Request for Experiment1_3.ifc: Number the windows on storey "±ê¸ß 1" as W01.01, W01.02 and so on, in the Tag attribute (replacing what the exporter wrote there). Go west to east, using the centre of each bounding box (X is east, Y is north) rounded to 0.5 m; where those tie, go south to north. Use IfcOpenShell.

First a look at what the model holds.

```python
import ifcopenshell
import ifcopenshell.util.element
import ifcopenshell.util.placement

model = ifcopenshell.open("Experiment1_3.ifc")
print(model.schema)
storey = next(s for s in model.by_type("IfcBuildingStorey") if s.Name == "±ê¸ß 1")
windows = [e for e in ifcopenshell.util.element.get_decomposition(storey) if e.is_a("IfcWindow")]
for e in sorted(windows, key=lambda e: e.id()):
    origin = ifcopenshell.util.placement.get_local_placement(e.ObjectPlacement)[:3, 3]
    print(e.id(), e.Tag, e.Name, origin.round(2) + 0.0, sep=" | ")
```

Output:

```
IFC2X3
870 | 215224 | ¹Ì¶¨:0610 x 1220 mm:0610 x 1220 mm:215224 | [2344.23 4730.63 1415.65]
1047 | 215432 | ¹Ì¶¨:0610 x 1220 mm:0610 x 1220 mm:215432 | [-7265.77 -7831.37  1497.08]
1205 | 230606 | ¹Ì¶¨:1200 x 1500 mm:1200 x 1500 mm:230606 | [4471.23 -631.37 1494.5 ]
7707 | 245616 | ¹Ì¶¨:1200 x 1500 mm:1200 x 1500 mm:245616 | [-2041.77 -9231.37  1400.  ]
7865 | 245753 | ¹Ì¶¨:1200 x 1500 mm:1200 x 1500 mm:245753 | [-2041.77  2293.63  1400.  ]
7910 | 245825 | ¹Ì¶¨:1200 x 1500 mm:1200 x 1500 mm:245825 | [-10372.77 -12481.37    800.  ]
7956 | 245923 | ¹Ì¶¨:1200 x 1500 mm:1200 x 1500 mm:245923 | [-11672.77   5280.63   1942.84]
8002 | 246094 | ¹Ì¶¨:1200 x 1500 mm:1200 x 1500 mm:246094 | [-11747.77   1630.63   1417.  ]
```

```python
import ifcopenshell
import ifcopenshell.geom
import ifcopenshell.util.element
import ifcopenshell.util.shape

model = ifcopenshell.open("Experiment1_3.ifc")
settings = ifcopenshell.geom.settings()
settings.set("use-world-coords", True)


def centre(element):
    shape = ifcopenshell.geom.create_shape(settings, element)
    return ifcopenshell.util.shape.get_bbox_centroid(shape.geometry)


storey = next(s for s in model.by_type("IfcBuildingStorey") if s.Name == "±ê¸ß 1")
windows = [e for e in ifcopenshell.util.element.get_decomposition(storey) if e.is_a("IfcWindow")]

# Insertion points can sit at a corner or the storey origin, so sort by the geometry (in metres).
centres = {e: centre(e) for e in windows}
windows.sort(key=lambda e: (round(centres[e][0] / 0.5), centres[e][1]))

for i, e in enumerate(windows, start=1):
    number = f"W01.{i:02d}"
    e.Tag = number
    print(e.id(), number)

model.write("Experiment1_3_updated.ifc")
```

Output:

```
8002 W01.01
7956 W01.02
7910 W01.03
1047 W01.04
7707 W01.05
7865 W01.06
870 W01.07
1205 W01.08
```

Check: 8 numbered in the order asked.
